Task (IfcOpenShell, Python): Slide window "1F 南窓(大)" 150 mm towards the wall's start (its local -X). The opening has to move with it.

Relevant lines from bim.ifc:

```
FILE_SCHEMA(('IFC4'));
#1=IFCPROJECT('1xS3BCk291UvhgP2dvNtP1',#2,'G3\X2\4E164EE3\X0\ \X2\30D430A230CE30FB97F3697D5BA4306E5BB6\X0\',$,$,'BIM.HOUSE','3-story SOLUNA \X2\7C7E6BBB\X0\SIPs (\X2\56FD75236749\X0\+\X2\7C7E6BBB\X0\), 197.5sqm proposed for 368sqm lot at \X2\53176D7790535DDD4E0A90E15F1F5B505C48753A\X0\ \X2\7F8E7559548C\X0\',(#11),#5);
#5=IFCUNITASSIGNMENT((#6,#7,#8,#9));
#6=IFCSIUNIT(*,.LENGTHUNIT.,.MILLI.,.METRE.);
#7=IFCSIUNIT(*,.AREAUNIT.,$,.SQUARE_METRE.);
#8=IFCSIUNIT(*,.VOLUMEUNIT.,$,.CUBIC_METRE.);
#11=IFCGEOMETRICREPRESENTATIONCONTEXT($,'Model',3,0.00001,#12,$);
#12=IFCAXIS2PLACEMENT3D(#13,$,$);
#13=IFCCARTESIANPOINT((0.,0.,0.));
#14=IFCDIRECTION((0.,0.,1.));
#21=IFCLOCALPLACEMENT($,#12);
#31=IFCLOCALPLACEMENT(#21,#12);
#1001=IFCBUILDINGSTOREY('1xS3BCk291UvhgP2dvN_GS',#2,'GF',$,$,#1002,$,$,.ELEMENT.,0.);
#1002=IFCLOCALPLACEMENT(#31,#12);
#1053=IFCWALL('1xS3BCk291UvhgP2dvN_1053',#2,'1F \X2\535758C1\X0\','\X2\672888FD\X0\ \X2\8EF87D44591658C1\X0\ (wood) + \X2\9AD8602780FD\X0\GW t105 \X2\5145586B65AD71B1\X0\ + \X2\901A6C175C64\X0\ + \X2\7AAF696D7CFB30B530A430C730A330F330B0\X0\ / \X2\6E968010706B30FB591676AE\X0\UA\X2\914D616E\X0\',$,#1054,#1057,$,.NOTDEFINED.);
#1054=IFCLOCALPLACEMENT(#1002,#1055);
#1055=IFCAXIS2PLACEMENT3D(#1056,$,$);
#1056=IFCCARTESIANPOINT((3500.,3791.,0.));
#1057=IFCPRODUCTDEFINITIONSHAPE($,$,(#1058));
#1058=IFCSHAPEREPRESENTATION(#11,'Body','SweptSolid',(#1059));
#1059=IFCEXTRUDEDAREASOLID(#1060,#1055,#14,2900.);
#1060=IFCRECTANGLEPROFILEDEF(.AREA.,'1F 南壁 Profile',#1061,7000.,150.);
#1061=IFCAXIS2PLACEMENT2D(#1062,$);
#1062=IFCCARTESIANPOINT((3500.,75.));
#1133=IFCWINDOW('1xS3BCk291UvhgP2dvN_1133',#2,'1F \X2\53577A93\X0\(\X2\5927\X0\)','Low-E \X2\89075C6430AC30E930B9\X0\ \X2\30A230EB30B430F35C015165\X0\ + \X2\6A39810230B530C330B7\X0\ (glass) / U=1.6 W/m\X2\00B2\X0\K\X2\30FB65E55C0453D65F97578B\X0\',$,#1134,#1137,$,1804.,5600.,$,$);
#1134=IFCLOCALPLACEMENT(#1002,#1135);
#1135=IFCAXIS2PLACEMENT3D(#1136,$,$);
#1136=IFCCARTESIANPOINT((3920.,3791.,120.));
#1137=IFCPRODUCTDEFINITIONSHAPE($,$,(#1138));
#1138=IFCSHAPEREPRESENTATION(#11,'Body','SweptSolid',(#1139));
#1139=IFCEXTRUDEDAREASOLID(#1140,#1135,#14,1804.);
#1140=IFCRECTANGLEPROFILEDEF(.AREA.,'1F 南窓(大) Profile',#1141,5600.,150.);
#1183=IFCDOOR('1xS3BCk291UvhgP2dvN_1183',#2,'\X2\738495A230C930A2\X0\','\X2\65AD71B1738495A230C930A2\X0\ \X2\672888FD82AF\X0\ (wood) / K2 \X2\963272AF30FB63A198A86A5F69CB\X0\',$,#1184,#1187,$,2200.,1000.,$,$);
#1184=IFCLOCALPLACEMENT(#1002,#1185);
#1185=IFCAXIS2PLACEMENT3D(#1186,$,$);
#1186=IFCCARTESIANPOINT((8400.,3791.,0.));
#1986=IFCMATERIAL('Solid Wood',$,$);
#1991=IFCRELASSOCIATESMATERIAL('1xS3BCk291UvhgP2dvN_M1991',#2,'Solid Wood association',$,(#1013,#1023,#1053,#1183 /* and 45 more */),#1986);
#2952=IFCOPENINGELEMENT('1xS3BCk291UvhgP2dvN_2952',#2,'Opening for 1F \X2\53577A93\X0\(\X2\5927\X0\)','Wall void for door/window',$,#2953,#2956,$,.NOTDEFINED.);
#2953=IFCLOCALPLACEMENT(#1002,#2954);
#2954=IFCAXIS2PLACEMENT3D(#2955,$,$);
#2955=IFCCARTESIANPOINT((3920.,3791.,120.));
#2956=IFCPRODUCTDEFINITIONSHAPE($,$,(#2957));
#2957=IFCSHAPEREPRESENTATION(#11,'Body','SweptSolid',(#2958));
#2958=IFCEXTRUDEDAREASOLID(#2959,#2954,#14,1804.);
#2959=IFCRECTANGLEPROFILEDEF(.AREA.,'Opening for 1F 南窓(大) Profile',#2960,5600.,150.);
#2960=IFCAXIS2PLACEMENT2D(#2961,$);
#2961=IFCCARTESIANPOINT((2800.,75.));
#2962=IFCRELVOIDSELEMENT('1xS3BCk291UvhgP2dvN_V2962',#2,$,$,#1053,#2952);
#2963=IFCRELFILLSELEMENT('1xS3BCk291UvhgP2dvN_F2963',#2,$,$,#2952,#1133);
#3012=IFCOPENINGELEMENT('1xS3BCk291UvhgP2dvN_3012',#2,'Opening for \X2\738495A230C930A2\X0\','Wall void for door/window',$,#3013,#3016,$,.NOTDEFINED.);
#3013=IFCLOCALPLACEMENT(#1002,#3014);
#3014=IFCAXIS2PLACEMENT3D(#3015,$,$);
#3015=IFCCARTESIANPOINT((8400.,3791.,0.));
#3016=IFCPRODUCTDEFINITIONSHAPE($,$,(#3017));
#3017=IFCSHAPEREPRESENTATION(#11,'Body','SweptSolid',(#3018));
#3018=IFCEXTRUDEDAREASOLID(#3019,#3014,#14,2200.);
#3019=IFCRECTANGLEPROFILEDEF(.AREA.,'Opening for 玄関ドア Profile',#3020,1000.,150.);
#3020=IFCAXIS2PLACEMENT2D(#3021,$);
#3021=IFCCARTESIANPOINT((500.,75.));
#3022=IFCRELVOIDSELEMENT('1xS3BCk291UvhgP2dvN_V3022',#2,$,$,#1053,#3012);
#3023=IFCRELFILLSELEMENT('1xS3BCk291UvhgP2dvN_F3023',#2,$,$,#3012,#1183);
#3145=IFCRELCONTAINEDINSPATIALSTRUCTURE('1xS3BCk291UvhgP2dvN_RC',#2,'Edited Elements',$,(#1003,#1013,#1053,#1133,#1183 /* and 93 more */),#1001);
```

```python
import ifcopenshell
import ifcopenshell.api.geometry
import ifcopenshell.util.placement

model = ifcopenshell.open("bim.ifc")

window = model.by_id(1133)
opening = window.FillsVoids[0].RelatingOpeningElement
wall = opening.VoidsElements[0].RelatingBuildingElement

wall_matrix = ifcopenshell.util.placement.get_local_placement(wall.ObjectPlacement)
shift = wall_matrix[:3, 0] * -150.0
before = ifcopenshell.util.placement.get_local_placement(window.ObjectPlacement)[:3, 3].copy()

# The window is not placed relative to its opening, so move both.
for product in (opening, window):
    matrix = ifcopenshell.util.placement.get_local_placement(product.ObjectPlacement)
    matrix[:3, 3] += shift
    ifcopenshell.api.geometry.edit_object_placement(model, product=product, matrix=matrix, is_si=False)

after = ifcopenshell.util.placement.get_local_placement(window.ObjectPlacement)[:3, 3]
print("window moved by", (after - before).round(3) + 0.0)

model.write("bim-out.ifc")
```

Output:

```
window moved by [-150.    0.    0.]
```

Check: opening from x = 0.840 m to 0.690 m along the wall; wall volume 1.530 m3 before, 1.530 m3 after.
